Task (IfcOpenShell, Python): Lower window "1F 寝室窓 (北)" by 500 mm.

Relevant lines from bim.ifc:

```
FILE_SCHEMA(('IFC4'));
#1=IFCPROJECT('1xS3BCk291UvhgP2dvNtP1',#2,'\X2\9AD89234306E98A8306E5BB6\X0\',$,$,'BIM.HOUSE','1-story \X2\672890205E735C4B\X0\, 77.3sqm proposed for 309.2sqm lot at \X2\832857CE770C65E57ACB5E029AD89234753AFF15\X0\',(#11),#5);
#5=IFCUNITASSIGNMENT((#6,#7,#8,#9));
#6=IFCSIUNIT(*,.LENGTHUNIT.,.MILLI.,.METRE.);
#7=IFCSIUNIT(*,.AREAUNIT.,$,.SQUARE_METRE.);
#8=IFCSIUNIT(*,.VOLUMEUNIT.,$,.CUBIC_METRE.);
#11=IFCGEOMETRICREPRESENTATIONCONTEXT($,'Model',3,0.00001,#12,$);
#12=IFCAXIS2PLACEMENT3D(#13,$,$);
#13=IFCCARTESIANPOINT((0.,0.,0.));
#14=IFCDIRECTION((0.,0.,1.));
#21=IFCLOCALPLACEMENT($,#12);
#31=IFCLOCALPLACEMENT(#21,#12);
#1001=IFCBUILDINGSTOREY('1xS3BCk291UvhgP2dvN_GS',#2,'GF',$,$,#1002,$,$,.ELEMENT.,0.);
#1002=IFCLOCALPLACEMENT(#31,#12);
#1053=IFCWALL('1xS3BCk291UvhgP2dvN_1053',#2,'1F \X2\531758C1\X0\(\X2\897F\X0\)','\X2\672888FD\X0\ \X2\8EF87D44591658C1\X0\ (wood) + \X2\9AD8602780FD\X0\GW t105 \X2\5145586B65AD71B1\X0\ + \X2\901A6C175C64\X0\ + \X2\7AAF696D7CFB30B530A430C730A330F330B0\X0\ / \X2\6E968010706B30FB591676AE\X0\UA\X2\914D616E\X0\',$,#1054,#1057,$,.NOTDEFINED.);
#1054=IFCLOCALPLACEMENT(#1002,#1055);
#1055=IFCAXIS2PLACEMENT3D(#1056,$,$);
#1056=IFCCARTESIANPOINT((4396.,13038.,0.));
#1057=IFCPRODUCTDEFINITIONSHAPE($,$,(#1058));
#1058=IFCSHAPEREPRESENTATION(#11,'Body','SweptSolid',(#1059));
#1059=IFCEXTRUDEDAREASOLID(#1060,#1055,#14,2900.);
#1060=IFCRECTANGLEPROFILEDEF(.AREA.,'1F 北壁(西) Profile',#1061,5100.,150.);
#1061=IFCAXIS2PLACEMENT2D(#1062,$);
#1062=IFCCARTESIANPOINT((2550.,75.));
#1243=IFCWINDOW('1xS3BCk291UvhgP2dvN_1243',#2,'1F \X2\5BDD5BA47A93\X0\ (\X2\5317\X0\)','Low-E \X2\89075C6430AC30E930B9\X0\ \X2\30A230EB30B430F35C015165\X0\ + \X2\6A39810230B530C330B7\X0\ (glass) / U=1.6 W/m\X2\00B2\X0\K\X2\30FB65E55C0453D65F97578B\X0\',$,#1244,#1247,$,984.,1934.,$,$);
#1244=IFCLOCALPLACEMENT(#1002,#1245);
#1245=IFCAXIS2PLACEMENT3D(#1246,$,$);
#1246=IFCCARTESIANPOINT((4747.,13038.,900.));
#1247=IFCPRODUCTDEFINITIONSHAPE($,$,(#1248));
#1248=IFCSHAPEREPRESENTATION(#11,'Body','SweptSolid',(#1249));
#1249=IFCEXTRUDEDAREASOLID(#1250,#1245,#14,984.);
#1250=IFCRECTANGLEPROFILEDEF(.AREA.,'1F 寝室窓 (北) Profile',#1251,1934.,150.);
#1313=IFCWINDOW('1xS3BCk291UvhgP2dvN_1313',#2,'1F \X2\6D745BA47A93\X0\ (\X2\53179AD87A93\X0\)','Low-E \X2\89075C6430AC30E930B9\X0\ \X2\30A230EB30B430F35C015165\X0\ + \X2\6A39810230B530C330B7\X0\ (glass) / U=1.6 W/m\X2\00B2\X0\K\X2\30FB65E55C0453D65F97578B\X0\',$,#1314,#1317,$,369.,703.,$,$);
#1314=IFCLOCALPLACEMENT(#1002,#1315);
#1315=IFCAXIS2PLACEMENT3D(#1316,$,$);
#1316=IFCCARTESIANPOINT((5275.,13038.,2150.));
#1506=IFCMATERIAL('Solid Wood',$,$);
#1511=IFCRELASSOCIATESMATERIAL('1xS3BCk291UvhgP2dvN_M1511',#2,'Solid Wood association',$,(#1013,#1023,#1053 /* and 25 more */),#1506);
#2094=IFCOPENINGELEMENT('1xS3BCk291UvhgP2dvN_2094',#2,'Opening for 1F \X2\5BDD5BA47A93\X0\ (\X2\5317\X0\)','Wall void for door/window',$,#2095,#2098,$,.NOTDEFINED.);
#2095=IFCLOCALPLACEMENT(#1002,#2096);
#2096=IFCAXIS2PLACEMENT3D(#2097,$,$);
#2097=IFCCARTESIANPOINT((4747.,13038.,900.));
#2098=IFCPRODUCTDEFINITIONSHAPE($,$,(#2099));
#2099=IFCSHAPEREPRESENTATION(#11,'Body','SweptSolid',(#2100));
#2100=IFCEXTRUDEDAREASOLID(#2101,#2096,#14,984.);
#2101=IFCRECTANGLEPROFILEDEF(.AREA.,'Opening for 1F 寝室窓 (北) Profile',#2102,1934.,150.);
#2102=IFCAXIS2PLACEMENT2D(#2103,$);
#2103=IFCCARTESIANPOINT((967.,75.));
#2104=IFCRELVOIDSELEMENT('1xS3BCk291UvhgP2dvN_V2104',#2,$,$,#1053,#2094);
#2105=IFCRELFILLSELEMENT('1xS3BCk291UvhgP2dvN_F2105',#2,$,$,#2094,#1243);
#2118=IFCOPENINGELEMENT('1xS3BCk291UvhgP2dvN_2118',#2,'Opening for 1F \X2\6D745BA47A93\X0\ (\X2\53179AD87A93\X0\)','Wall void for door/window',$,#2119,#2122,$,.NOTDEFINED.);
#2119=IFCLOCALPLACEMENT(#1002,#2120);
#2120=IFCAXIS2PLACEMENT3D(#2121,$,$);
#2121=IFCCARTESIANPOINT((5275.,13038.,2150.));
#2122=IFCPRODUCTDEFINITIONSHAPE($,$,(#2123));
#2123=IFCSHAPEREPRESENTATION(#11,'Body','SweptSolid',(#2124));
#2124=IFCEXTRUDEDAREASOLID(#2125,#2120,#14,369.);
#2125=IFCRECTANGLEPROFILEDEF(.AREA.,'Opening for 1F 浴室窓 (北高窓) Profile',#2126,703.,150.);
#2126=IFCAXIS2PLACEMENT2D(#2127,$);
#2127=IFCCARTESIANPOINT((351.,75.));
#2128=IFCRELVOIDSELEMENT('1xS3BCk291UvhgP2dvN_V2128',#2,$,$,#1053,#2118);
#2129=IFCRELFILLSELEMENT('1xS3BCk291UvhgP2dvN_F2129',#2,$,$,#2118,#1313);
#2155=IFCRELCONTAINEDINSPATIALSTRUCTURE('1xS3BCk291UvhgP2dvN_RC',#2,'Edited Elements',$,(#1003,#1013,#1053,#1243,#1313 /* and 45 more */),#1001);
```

```python
import numpy as np
import ifcopenshell
import ifcopenshell.api.geometry
import ifcopenshell.util.placement
import ifcopenshell.util.unit

model = ifcopenshell.open("bim.ifc")
unit_scale = ifcopenshell.util.unit.calculate_unit_scale(model)

window = model.by_id(1243)
opening = window.FillsVoids[0].RelatingOpeningElement
dz = -0.5 / unit_scale

shift = np.array([0.0, 0.0, dz])
# The window is not placed relative to its opening, so move both.
for product in (opening, window):
    matrix = ifcopenshell.util.placement.get_local_placement(product.ObjectPlacement)
    matrix[:3, 3] += shift
    ifcopenshell.api.geometry.edit_object_placement(model, product=product, matrix=matrix, is_si=False)

print(f"moved by {dz * unit_scale:+.3f} m")

model.write("bim-out.ifc")
```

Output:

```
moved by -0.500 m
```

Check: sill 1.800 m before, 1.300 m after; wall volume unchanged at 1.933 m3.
